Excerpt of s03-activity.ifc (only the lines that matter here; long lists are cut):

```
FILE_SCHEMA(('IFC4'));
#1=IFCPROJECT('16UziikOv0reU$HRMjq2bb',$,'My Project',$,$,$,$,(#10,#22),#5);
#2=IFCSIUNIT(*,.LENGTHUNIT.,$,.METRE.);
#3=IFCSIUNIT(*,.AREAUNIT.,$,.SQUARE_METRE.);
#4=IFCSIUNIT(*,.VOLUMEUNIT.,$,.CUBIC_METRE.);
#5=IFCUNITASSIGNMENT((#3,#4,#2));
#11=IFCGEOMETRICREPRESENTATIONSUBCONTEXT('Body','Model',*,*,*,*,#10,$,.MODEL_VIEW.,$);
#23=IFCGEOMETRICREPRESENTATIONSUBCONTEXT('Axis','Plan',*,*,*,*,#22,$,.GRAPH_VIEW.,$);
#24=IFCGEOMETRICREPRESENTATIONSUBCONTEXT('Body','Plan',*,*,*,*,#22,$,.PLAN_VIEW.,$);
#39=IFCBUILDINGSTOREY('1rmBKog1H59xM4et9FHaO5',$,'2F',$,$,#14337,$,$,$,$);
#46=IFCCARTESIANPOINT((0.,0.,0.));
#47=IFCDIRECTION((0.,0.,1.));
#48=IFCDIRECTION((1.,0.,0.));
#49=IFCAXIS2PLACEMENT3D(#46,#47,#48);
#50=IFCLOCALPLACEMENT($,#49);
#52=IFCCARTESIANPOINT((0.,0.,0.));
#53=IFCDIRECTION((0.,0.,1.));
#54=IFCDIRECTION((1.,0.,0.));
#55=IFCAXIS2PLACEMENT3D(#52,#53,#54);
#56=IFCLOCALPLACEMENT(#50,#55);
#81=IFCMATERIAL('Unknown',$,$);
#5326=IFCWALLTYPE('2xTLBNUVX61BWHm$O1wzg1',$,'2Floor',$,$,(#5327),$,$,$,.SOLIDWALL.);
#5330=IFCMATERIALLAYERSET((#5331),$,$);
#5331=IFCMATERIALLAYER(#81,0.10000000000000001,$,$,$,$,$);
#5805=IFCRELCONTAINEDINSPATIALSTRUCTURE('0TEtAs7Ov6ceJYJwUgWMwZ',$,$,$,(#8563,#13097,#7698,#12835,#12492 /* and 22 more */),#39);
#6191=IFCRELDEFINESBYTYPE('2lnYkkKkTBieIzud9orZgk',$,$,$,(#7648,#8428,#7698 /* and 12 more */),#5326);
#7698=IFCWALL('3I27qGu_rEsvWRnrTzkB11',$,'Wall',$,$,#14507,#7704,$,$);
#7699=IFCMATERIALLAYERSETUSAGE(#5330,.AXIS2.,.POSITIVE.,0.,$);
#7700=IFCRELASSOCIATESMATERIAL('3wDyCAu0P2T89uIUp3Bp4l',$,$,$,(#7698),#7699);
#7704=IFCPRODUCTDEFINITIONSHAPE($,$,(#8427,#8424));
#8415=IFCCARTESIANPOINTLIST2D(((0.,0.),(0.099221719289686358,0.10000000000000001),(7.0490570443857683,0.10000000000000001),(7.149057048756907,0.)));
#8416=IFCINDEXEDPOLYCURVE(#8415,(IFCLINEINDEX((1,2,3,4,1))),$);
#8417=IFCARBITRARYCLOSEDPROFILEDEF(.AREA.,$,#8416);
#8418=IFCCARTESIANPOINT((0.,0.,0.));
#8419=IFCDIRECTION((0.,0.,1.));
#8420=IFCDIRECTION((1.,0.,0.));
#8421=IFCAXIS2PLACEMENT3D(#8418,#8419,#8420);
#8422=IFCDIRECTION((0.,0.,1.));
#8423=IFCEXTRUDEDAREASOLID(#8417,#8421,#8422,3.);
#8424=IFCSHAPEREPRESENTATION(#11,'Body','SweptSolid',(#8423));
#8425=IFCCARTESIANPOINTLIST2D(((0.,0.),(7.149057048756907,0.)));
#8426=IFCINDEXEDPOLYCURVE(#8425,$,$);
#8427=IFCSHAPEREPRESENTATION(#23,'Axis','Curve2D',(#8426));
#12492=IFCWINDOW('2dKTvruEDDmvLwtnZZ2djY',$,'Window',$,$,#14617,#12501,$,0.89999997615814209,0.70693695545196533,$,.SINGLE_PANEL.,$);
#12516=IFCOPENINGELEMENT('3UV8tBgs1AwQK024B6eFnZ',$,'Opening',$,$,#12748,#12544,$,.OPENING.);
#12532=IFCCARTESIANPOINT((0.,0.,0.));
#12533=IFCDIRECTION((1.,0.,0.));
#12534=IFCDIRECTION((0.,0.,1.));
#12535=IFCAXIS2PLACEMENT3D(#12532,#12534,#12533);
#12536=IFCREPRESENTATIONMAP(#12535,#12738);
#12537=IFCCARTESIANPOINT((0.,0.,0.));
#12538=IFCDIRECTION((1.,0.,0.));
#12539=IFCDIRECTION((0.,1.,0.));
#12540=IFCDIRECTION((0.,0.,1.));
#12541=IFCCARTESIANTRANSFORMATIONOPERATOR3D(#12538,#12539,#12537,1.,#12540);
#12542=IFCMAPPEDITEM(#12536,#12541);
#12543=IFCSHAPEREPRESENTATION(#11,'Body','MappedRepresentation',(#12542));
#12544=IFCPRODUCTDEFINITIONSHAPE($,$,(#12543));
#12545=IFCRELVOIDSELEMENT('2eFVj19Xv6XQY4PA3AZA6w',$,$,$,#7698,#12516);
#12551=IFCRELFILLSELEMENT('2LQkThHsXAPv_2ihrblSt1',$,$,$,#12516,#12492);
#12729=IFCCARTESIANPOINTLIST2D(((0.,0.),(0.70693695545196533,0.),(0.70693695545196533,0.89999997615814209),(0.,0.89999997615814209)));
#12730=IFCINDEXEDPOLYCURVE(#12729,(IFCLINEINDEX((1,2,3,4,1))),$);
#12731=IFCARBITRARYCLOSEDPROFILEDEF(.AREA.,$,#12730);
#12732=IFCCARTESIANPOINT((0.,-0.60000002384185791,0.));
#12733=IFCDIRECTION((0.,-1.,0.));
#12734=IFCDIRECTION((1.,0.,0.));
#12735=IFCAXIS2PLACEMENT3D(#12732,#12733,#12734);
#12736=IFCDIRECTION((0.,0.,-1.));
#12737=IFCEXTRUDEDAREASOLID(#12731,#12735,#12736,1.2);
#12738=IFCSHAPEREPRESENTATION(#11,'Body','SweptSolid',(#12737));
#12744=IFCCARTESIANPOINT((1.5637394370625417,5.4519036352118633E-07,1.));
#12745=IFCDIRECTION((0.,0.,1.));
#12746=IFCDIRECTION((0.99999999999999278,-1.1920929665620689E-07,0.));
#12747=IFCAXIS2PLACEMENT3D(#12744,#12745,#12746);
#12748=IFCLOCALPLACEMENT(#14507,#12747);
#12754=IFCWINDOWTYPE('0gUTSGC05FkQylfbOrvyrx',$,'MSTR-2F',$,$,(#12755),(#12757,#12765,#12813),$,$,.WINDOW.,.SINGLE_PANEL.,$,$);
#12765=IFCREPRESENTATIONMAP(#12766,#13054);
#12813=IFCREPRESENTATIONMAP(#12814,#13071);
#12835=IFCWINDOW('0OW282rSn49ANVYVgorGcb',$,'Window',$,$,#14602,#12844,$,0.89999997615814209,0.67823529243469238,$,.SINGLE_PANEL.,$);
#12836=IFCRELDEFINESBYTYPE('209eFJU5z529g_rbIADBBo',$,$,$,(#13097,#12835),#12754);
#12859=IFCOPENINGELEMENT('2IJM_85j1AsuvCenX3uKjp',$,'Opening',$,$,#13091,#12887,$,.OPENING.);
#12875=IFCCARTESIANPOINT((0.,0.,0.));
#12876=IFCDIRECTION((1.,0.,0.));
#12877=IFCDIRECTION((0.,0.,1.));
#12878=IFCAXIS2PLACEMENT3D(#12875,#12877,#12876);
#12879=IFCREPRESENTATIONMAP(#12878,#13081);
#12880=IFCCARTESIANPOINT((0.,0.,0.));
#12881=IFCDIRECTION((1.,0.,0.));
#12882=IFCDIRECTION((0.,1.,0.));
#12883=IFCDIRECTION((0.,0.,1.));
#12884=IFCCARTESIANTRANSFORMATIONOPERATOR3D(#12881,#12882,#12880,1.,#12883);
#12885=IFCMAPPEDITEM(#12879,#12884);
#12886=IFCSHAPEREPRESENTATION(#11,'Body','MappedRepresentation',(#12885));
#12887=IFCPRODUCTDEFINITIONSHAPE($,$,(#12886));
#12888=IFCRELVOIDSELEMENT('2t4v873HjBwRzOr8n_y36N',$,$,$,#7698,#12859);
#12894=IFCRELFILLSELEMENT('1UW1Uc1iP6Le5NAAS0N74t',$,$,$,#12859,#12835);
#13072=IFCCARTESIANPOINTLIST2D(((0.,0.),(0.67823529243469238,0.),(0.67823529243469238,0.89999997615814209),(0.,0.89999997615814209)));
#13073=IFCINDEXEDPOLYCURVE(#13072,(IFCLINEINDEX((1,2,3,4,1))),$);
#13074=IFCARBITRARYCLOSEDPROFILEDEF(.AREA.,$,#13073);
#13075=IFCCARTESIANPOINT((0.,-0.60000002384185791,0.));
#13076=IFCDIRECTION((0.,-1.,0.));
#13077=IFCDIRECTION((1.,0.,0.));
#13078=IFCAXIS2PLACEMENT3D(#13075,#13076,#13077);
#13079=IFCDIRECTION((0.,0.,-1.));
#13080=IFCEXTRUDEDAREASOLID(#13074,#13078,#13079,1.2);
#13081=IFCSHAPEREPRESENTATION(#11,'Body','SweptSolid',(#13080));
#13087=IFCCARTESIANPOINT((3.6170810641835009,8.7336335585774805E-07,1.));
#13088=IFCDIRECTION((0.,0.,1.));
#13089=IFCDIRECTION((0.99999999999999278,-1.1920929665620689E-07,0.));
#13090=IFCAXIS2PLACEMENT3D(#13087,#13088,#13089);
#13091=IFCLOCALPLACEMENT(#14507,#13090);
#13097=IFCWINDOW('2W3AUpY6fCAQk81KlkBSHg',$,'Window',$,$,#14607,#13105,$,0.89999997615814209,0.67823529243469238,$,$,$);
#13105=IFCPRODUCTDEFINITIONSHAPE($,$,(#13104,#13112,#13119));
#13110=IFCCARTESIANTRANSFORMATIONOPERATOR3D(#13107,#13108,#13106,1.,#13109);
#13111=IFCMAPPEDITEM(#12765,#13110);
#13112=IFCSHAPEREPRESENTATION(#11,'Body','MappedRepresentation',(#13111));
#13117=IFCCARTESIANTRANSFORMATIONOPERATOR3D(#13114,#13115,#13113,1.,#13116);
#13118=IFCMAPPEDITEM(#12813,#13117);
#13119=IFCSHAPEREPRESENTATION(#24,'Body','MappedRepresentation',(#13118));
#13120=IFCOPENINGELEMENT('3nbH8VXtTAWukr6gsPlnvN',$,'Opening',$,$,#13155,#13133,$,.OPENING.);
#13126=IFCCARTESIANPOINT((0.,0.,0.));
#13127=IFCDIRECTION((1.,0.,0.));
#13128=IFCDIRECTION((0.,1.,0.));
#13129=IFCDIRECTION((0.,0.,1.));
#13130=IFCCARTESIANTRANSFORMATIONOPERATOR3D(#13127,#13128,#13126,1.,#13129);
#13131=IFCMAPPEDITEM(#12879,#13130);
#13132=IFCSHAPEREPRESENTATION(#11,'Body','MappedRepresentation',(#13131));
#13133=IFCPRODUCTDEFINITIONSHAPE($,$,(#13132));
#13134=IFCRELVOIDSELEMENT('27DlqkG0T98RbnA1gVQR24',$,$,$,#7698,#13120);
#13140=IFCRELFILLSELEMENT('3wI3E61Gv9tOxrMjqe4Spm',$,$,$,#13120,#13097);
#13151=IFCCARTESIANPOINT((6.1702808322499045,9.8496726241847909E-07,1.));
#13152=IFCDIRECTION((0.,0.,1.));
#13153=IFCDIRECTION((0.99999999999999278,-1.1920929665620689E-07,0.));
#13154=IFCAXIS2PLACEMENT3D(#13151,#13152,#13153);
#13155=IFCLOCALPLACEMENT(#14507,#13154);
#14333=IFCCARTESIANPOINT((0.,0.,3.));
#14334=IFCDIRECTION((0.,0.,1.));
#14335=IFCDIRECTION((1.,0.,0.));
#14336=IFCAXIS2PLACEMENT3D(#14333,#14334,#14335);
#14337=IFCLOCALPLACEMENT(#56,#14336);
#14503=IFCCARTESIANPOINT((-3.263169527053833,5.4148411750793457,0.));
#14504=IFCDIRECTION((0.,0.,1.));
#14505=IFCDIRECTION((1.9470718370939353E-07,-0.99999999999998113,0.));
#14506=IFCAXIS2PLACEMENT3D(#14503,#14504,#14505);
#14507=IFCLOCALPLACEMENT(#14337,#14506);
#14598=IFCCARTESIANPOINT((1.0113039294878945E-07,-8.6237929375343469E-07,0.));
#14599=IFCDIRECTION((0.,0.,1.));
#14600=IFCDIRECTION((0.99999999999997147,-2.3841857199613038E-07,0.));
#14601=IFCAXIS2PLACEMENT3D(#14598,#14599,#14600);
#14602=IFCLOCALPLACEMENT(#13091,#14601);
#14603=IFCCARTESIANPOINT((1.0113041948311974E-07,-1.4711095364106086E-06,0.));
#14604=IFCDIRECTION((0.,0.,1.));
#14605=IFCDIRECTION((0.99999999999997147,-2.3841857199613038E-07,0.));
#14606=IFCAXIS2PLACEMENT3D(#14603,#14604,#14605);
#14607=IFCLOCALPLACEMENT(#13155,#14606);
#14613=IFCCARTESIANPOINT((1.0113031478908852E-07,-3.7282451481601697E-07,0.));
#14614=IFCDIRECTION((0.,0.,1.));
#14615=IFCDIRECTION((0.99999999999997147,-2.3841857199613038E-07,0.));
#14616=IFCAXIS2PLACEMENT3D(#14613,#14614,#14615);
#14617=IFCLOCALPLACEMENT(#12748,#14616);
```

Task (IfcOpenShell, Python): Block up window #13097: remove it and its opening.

```python
import ifcopenshell
import ifcopenshell.api.feature
import ifcopenshell.api.root
import ifcopenshell.geom
import ifcopenshell.util.shape

model = ifcopenshell.open("s03-activity.ifc")
settings = ifcopenshell.geom.settings()


def volume(element):
    """Net volume in cubic metres, openings subtracted."""
    shape = ifcopenshell.geom.create_shape(settings, element)
    return ifcopenshell.util.shape.get_volume(shape.geometry)


window = model.by_guid("2W3AUpY6fCAQk81KlkBSHg")
opening = window.FillsVoids[0].RelatingOpeningElement
wall = opening.VoidsElements[0].RelatingBuildingElement
before = volume(wall)

ifcopenshell.api.root.remove_product(model, product=window)
ifcopenshell.api.feature.remove_feature(model, feature=opening)

after = volume(wall)

print(f"wall volume {before:.3f} -> {after:.3f} m3")

model.write("s03-activity_updated.ifc")
```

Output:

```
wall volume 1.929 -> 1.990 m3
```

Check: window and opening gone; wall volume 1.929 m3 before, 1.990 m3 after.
